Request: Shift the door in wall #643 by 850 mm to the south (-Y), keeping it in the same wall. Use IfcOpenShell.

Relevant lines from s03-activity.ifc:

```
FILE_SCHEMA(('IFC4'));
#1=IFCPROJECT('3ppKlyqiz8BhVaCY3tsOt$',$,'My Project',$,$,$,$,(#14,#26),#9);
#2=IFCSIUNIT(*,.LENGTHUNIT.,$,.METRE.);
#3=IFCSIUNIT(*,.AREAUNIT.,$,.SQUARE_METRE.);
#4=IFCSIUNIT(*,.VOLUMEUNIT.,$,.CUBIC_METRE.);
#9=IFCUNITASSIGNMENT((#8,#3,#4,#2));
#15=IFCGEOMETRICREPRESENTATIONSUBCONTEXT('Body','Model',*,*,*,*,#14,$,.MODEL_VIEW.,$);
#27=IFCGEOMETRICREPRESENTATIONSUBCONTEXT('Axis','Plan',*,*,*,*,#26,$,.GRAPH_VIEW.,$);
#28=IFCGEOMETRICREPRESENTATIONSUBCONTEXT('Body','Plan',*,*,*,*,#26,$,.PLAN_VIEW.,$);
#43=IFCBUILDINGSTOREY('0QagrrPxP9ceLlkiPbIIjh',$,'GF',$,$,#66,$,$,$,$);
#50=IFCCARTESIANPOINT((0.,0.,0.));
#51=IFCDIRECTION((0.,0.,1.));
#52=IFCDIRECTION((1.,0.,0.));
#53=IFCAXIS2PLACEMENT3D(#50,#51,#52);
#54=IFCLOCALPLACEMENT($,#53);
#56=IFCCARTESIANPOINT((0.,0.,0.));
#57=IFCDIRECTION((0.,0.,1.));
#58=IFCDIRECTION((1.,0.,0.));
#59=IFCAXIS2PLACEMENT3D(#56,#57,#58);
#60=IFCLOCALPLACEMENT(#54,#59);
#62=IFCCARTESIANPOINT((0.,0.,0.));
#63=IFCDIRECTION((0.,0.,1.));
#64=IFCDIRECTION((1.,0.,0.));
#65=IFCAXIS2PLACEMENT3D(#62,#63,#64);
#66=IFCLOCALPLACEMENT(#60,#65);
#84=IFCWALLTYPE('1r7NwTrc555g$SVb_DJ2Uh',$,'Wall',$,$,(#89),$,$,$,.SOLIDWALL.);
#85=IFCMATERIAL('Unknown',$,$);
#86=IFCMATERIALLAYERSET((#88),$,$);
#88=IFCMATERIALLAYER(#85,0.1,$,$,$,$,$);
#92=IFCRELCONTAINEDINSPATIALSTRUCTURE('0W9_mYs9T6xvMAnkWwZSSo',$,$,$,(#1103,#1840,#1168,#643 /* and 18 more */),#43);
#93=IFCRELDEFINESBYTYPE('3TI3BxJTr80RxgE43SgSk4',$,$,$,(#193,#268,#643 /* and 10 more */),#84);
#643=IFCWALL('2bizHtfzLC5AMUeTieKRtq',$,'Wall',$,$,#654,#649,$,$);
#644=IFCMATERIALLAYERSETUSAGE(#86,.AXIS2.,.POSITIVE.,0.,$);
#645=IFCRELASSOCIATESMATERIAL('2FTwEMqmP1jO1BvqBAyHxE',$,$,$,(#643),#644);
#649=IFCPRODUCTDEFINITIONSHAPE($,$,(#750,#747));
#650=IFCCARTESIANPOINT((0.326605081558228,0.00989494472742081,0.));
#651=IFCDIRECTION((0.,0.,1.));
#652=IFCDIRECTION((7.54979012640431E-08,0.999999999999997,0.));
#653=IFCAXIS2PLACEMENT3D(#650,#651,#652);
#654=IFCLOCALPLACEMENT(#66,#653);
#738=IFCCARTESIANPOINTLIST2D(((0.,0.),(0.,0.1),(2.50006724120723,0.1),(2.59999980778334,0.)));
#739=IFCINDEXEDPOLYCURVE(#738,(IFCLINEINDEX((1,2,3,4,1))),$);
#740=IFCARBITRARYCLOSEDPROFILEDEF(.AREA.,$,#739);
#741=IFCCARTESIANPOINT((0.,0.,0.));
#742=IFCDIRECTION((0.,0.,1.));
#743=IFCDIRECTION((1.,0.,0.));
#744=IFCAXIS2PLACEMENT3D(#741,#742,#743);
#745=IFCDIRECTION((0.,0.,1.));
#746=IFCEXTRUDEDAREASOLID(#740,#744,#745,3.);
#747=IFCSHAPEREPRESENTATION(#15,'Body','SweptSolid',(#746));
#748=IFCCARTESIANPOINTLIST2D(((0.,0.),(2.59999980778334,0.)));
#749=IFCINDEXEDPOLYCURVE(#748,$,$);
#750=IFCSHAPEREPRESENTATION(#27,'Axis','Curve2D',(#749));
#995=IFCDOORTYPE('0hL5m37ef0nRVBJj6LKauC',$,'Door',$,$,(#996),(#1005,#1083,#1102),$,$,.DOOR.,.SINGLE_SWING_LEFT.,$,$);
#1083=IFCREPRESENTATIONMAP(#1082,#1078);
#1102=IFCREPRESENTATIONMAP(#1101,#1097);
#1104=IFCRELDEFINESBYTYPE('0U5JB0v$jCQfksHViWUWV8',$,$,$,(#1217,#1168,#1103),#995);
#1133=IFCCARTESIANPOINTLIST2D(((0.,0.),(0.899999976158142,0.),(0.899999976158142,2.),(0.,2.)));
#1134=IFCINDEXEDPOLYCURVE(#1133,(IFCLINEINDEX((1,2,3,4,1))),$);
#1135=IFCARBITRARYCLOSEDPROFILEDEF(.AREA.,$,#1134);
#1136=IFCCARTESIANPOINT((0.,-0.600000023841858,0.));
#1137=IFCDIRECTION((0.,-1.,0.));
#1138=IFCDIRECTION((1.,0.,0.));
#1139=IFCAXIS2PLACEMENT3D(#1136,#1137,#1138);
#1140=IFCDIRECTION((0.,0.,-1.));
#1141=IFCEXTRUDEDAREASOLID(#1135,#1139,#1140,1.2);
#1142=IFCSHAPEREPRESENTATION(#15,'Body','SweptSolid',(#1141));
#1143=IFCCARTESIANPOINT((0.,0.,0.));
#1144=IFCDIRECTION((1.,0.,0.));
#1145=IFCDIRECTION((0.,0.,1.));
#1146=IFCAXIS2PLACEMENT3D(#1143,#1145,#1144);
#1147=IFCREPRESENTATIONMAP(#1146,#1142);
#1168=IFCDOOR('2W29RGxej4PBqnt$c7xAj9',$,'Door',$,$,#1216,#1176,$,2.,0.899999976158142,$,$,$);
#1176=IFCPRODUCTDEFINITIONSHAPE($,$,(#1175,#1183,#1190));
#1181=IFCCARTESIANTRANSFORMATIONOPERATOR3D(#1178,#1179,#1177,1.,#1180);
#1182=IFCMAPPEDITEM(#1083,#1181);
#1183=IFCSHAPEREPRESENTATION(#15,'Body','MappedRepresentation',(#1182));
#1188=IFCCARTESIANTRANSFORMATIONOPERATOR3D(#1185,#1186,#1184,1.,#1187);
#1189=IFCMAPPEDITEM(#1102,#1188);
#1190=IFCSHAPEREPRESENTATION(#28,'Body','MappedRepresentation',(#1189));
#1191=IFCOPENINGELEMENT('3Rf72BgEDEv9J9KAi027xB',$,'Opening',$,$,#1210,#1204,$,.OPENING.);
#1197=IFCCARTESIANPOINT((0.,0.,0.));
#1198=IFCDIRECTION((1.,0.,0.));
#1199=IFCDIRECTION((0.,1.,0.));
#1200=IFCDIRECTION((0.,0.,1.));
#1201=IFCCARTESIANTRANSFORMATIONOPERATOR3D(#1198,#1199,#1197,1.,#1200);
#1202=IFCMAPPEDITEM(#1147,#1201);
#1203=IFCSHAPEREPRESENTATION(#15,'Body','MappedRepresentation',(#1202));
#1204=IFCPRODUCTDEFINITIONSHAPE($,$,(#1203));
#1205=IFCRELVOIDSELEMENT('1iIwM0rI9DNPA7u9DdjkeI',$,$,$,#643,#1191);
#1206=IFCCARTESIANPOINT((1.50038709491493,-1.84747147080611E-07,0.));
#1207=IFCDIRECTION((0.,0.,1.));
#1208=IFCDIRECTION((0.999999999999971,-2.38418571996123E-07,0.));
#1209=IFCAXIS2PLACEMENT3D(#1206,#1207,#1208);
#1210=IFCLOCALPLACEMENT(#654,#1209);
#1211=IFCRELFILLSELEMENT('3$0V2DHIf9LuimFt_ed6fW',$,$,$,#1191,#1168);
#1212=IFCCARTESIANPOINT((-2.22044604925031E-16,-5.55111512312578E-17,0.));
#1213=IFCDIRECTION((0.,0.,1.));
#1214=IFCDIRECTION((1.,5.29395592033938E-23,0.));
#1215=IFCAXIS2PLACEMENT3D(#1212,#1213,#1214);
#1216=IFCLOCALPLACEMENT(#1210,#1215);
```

```python
import ifcopenshell
import ifcopenshell.api.geometry
import ifcopenshell.util.placement
import ifcopenshell.util.unit

model = ifcopenshell.open("s03-activity.ifc")
unit_scale = ifcopenshell.util.unit.calculate_unit_scale(model)

door = model.by_id(1168)
opening = door.FillsVoids[0].RelatingOpeningElement
wall = opening.VoidsElements[0].RelatingBuildingElement

wall_matrix = ifcopenshell.util.placement.get_local_placement(wall.ObjectPlacement)
shift = wall_matrix[:3, 0] * -0.85 / unit_scale
before = ifcopenshell.util.placement.get_local_placement(door.ObjectPlacement)[:3, 3].copy()

# The door is placed relative to its opening, so it follows when the opening moves.
matrix = ifcopenshell.util.placement.get_local_placement(opening.ObjectPlacement)
matrix[:3, 3] += shift
ifcopenshell.api.geometry.edit_object_placement(
    model, product=opening, matrix=matrix, is_si=False, should_transform_children=True
)

after = ifcopenshell.util.placement.get_local_placement(door.ObjectPlacement)[:3, 3]
print("door moved by", (after - before).round(3) + 0.0)

model.write("s03-activity_edited.ifc")
```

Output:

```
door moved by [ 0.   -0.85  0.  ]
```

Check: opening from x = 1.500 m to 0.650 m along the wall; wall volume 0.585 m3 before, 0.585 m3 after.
